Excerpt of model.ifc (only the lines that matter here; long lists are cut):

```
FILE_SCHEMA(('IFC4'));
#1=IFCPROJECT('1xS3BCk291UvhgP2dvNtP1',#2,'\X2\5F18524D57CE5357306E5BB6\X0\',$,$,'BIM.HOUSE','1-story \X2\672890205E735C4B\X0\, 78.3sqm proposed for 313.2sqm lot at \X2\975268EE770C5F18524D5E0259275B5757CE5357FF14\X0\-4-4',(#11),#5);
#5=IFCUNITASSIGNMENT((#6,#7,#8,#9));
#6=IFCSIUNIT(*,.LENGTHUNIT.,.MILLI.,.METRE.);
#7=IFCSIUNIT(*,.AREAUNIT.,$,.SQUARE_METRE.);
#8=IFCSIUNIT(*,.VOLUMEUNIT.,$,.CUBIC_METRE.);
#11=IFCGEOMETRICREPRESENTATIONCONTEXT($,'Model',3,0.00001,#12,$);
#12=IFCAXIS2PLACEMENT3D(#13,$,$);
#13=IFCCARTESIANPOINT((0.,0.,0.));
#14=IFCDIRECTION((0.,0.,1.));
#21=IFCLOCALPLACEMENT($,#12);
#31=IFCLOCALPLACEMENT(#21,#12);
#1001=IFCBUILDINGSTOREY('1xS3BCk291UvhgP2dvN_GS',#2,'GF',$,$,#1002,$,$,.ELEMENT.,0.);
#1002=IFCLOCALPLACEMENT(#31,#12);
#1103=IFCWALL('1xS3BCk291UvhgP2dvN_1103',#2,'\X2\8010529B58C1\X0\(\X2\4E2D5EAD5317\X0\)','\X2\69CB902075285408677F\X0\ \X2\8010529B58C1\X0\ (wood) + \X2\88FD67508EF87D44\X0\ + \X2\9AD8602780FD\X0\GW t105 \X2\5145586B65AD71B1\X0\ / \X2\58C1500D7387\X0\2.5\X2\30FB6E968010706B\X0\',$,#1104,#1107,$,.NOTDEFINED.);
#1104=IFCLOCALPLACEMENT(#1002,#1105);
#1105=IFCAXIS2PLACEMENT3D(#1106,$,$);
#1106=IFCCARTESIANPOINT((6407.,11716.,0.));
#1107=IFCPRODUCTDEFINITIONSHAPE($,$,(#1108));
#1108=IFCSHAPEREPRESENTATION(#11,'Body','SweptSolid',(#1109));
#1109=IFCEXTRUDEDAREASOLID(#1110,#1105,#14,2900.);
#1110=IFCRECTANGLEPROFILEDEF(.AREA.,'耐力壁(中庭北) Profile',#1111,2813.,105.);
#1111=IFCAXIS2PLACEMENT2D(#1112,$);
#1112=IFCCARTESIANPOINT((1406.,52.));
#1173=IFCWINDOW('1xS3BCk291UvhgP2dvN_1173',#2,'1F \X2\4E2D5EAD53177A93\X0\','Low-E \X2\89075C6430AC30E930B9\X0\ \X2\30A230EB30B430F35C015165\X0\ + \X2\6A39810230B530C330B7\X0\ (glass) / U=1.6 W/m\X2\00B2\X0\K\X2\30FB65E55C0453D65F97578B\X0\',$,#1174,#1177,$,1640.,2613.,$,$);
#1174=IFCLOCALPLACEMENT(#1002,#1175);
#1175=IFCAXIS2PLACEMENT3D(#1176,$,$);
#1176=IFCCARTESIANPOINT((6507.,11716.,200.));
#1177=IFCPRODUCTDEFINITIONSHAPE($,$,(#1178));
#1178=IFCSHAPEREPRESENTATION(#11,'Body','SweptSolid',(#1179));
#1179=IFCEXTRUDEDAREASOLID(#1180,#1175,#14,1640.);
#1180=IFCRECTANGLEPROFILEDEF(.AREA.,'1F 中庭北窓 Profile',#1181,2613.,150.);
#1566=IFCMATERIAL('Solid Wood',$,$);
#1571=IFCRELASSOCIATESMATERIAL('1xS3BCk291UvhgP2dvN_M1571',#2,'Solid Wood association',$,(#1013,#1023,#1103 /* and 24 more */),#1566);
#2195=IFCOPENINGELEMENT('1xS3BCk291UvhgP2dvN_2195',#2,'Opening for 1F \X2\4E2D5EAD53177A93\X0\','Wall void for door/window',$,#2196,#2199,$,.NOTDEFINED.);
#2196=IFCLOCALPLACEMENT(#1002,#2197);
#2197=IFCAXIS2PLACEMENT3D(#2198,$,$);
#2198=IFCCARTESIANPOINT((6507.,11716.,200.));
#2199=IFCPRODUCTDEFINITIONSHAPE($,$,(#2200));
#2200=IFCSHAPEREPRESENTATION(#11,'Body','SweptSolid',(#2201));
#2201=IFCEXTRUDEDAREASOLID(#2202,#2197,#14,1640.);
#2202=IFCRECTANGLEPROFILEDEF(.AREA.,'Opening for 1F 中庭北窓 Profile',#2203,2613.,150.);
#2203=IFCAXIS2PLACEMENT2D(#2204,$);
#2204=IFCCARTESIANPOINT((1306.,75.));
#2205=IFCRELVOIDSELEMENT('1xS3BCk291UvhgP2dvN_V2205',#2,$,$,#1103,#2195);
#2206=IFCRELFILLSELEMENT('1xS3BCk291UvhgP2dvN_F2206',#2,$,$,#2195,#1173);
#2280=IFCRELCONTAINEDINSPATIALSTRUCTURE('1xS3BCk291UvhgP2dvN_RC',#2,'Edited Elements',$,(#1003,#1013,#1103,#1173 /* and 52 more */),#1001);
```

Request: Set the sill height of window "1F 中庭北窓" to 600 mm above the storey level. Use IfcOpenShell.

```python
import numpy as np
import ifcopenshell
import ifcopenshell.api.geometry
import ifcopenshell.geom
import ifcopenshell.util.element
import ifcopenshell.util.placement
import ifcopenshell.util.shape
import ifcopenshell.util.unit

model = ifcopenshell.open("model.ifc")
unit_scale = ifcopenshell.util.unit.calculate_unit_scale(model)

window = model.by_guid("1xS3BCk291UvhgP2dvN_1173")
opening = window.FillsVoids[0].RelatingOpeningElement
storey = ifcopenshell.util.element.get_container(window, ifc_class="IfcBuildingStorey")
level = ifcopenshell.util.placement.get_local_placement(storey.ObjectPlacement)[2, 3]

# The opening's origin need not be at the sill, so measure its lowest point.
shape = ifcopenshell.geom.create_shape(ifcopenshell.geom.settings(), opening)
bottom = ifcopenshell.util.shape.get_shape_bottom_elevation(shape, shape.geometry) / unit_scale
dz = level + 0.6 / unit_scale - bottom

shift = np.array([0.0, 0.0, dz])
# The window is not placed relative to its opening, so move both.
for product in (opening, window):
    matrix = ifcopenshell.util.placement.get_local_placement(product.ObjectPlacement)
    matrix[:3, 3] += shift
    ifcopenshell.api.geometry.edit_object_placement(model, product=product, matrix=matrix, is_si=False)

print(f"moved by {dz * unit_scale:+.3f} m")

model.write("model_rev.ifc")
```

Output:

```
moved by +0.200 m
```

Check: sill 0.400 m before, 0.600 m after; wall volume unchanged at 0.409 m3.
